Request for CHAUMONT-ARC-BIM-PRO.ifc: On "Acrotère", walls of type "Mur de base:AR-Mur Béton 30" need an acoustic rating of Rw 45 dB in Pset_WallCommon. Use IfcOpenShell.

First a look at what the model holds.

```python
import ifcopenshell
import ifcopenshell.util.element

model = ifcopenshell.open("CHAUMONT-ARC-BIM-PRO.ifc")
print(model.schema)
storey = next(s for s in model.by_type("IfcBuildingStorey") if s.Name == "Acrotère")
walls = [e for e in ifcopenshell.util.element.get_decomposition(storey) if e.is_a("IfcWall")]
seen = {}
for e in walls:
    element_type = ifcopenshell.util.element.get_type(e)
    key = (element_type.Name if element_type != e and element_type else None, ifcopenshell.util.element.get_pset(e, "Pset_WallCommon", "AcousticRating"))
    seen[key] = seen.get(key, 0) + 1
for (name, value), count in sorted(seen.items(), key=str):
    print(count, "x", name, "|", value)
```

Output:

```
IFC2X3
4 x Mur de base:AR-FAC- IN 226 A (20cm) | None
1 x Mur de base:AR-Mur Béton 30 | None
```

```python
import ifcopenshell
import ifcopenshell.api.pset
import ifcopenshell.util.element

model = ifcopenshell.open("CHAUMONT-ARC-BIM-PRO.ifc")

storey = next(s for s in model.by_type("IfcBuildingStorey") if s.Name == "Acrotère")
walls = [e for e in ifcopenshell.util.element.get_decomposition(storey) if e.is_a("IfcWall")]

count = 0
for e in walls:
    element_type = ifcopenshell.util.element.get_type(e)
    if element_type in (None, e) or element_type.Name != "Mur de base:AR-Mur Béton 30":
        continue
    # add_pset returns the element's existing set when there is one.
    pset = ifcopenshell.api.pset.add_pset(model, product=e, name="Pset_WallCommon")
    ifcopenshell.api.pset.edit_pset(model, pset=pset, properties={"AcousticRating": "Rw 45 dB"})
    count += 1

print(count, "walls updated")

model.write("CHAUMONT-ARC-BIM-PRO_updated.ifc")
```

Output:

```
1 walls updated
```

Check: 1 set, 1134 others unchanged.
